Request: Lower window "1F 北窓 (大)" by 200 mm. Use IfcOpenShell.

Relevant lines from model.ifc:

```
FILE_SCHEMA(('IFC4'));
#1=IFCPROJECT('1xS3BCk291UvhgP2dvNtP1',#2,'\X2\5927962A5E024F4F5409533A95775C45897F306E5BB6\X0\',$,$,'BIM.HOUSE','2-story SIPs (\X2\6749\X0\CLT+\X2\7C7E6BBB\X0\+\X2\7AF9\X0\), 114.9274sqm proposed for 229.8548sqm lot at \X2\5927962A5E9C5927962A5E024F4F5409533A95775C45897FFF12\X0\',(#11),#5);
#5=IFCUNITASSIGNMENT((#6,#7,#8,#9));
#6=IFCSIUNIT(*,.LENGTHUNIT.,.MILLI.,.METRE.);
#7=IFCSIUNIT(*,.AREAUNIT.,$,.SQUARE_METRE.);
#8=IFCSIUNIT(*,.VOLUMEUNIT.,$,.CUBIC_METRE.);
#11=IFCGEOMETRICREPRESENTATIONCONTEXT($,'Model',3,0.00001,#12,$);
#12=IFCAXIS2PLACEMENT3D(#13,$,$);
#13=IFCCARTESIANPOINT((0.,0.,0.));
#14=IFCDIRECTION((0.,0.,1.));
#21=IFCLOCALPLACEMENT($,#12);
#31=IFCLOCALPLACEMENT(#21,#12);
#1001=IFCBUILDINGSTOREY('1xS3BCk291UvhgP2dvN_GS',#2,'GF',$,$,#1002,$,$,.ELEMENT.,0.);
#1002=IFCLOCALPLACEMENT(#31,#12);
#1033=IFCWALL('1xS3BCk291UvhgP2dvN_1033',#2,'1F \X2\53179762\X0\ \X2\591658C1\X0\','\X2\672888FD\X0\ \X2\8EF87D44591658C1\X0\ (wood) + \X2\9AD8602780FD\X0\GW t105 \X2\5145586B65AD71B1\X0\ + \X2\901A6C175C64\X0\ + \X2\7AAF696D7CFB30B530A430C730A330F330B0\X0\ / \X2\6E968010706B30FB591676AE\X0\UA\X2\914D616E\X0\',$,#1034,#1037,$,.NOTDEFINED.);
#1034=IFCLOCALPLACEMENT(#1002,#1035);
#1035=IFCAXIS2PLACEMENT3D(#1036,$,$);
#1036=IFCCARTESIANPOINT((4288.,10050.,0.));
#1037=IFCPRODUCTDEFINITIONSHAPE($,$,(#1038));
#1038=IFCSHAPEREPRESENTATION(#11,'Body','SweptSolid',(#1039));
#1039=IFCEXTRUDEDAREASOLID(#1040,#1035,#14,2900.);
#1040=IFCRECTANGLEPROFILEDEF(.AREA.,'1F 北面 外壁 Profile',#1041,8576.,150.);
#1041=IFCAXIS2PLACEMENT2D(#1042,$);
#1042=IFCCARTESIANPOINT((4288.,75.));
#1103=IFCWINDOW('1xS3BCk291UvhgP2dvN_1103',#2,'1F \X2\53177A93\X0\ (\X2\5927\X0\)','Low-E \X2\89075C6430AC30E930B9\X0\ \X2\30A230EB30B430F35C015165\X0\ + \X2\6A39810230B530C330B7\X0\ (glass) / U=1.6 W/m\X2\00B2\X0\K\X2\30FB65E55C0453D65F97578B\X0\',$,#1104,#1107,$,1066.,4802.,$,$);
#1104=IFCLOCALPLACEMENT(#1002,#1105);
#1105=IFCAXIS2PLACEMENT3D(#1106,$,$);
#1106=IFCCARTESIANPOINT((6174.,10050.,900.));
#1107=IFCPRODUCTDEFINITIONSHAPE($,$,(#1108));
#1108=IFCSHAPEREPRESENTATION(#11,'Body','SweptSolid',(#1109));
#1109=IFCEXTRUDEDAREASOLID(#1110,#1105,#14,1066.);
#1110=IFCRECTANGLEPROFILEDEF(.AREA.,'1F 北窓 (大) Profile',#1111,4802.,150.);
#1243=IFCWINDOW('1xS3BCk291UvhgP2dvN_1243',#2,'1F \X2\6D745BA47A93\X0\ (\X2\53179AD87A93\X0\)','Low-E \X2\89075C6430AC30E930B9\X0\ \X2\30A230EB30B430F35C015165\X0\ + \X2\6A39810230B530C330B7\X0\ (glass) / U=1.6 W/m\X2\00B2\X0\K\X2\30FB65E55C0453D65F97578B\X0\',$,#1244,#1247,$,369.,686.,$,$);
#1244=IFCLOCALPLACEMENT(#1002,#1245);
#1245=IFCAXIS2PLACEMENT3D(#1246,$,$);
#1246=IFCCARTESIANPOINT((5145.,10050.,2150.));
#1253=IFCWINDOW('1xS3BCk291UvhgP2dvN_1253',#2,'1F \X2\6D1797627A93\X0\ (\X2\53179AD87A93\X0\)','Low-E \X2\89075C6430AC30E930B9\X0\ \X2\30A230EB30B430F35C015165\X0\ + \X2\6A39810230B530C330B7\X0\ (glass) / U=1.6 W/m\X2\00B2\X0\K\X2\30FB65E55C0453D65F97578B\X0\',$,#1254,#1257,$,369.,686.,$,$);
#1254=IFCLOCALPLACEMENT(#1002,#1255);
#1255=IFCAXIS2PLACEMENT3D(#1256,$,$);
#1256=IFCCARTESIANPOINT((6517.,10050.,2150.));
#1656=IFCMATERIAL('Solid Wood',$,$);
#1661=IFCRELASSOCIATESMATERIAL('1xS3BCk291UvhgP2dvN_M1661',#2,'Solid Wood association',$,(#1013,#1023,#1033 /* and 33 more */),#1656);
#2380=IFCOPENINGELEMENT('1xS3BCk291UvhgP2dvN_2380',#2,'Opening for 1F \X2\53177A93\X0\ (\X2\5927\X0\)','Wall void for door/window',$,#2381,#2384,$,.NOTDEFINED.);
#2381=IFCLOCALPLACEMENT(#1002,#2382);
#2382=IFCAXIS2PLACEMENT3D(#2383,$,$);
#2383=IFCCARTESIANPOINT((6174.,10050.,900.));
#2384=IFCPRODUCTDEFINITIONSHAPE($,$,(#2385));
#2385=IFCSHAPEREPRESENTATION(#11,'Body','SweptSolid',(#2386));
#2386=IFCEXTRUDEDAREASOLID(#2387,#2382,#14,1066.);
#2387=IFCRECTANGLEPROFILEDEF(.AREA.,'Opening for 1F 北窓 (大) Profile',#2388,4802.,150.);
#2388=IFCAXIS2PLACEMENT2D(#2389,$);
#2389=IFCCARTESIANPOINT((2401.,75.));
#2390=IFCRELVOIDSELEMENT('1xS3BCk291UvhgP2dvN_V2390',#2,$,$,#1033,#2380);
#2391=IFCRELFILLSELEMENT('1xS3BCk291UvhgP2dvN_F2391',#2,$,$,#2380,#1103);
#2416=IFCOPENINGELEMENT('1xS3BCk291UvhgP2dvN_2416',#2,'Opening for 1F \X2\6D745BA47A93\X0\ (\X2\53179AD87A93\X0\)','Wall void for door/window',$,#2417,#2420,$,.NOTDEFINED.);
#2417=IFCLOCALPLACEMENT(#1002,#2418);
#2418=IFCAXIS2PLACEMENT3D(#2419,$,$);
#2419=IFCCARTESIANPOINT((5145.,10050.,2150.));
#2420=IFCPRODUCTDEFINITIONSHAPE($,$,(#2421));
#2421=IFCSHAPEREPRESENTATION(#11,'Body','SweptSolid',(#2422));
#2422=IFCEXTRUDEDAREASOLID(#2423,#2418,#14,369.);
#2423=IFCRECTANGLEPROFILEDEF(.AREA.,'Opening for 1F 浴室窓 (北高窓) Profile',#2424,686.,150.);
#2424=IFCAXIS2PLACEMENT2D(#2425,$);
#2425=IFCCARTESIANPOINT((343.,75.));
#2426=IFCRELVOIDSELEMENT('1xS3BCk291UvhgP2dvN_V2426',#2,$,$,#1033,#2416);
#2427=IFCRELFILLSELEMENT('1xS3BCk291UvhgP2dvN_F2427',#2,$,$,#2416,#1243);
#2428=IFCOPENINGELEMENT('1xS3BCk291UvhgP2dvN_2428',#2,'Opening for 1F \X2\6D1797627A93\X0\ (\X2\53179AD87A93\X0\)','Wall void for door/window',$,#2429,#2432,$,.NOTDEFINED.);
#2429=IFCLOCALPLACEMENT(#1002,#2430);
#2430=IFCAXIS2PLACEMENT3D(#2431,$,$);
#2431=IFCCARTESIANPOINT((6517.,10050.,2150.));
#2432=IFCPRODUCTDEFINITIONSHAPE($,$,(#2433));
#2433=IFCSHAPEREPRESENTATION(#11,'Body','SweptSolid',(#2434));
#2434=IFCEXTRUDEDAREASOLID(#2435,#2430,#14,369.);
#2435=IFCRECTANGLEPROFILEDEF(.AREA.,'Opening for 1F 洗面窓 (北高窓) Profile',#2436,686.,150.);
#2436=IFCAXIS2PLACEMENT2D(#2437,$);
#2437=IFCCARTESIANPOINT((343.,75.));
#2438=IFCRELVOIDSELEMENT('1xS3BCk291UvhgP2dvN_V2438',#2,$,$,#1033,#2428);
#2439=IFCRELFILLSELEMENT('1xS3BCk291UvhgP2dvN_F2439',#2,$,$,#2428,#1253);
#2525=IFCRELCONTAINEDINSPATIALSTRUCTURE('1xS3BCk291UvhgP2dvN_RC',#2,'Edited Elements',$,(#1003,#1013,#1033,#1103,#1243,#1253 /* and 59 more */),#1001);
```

```python
import numpy as np
import ifcopenshell
import ifcopenshell.api.geometry
import ifcopenshell.util.placement
import ifcopenshell.util.unit

model = ifcopenshell.open("model.ifc")
unit_scale = ifcopenshell.util.unit.calculate_unit_scale(model)

window = model.by_guid("1xS3BCk291UvhgP2dvN_1103")
opening = window.FillsVoids[0].RelatingOpeningElement
dz = -200.0

shift = np.array([0.0, 0.0, dz])
# The window is not placed relative to its opening, so move both.
for product in (opening, window):
    matrix = ifcopenshell.util.placement.get_local_placement(product.ObjectPlacement)
    matrix[:3, 3] += shift
    ifcopenshell.api.geometry.edit_object_placement(model, product=product, matrix=matrix, is_si=False)

print(f"moved by {dz * unit_scale:+.3f} m")

model.write("model_rev.ifc")
```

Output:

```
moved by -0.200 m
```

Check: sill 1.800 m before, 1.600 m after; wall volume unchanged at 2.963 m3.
